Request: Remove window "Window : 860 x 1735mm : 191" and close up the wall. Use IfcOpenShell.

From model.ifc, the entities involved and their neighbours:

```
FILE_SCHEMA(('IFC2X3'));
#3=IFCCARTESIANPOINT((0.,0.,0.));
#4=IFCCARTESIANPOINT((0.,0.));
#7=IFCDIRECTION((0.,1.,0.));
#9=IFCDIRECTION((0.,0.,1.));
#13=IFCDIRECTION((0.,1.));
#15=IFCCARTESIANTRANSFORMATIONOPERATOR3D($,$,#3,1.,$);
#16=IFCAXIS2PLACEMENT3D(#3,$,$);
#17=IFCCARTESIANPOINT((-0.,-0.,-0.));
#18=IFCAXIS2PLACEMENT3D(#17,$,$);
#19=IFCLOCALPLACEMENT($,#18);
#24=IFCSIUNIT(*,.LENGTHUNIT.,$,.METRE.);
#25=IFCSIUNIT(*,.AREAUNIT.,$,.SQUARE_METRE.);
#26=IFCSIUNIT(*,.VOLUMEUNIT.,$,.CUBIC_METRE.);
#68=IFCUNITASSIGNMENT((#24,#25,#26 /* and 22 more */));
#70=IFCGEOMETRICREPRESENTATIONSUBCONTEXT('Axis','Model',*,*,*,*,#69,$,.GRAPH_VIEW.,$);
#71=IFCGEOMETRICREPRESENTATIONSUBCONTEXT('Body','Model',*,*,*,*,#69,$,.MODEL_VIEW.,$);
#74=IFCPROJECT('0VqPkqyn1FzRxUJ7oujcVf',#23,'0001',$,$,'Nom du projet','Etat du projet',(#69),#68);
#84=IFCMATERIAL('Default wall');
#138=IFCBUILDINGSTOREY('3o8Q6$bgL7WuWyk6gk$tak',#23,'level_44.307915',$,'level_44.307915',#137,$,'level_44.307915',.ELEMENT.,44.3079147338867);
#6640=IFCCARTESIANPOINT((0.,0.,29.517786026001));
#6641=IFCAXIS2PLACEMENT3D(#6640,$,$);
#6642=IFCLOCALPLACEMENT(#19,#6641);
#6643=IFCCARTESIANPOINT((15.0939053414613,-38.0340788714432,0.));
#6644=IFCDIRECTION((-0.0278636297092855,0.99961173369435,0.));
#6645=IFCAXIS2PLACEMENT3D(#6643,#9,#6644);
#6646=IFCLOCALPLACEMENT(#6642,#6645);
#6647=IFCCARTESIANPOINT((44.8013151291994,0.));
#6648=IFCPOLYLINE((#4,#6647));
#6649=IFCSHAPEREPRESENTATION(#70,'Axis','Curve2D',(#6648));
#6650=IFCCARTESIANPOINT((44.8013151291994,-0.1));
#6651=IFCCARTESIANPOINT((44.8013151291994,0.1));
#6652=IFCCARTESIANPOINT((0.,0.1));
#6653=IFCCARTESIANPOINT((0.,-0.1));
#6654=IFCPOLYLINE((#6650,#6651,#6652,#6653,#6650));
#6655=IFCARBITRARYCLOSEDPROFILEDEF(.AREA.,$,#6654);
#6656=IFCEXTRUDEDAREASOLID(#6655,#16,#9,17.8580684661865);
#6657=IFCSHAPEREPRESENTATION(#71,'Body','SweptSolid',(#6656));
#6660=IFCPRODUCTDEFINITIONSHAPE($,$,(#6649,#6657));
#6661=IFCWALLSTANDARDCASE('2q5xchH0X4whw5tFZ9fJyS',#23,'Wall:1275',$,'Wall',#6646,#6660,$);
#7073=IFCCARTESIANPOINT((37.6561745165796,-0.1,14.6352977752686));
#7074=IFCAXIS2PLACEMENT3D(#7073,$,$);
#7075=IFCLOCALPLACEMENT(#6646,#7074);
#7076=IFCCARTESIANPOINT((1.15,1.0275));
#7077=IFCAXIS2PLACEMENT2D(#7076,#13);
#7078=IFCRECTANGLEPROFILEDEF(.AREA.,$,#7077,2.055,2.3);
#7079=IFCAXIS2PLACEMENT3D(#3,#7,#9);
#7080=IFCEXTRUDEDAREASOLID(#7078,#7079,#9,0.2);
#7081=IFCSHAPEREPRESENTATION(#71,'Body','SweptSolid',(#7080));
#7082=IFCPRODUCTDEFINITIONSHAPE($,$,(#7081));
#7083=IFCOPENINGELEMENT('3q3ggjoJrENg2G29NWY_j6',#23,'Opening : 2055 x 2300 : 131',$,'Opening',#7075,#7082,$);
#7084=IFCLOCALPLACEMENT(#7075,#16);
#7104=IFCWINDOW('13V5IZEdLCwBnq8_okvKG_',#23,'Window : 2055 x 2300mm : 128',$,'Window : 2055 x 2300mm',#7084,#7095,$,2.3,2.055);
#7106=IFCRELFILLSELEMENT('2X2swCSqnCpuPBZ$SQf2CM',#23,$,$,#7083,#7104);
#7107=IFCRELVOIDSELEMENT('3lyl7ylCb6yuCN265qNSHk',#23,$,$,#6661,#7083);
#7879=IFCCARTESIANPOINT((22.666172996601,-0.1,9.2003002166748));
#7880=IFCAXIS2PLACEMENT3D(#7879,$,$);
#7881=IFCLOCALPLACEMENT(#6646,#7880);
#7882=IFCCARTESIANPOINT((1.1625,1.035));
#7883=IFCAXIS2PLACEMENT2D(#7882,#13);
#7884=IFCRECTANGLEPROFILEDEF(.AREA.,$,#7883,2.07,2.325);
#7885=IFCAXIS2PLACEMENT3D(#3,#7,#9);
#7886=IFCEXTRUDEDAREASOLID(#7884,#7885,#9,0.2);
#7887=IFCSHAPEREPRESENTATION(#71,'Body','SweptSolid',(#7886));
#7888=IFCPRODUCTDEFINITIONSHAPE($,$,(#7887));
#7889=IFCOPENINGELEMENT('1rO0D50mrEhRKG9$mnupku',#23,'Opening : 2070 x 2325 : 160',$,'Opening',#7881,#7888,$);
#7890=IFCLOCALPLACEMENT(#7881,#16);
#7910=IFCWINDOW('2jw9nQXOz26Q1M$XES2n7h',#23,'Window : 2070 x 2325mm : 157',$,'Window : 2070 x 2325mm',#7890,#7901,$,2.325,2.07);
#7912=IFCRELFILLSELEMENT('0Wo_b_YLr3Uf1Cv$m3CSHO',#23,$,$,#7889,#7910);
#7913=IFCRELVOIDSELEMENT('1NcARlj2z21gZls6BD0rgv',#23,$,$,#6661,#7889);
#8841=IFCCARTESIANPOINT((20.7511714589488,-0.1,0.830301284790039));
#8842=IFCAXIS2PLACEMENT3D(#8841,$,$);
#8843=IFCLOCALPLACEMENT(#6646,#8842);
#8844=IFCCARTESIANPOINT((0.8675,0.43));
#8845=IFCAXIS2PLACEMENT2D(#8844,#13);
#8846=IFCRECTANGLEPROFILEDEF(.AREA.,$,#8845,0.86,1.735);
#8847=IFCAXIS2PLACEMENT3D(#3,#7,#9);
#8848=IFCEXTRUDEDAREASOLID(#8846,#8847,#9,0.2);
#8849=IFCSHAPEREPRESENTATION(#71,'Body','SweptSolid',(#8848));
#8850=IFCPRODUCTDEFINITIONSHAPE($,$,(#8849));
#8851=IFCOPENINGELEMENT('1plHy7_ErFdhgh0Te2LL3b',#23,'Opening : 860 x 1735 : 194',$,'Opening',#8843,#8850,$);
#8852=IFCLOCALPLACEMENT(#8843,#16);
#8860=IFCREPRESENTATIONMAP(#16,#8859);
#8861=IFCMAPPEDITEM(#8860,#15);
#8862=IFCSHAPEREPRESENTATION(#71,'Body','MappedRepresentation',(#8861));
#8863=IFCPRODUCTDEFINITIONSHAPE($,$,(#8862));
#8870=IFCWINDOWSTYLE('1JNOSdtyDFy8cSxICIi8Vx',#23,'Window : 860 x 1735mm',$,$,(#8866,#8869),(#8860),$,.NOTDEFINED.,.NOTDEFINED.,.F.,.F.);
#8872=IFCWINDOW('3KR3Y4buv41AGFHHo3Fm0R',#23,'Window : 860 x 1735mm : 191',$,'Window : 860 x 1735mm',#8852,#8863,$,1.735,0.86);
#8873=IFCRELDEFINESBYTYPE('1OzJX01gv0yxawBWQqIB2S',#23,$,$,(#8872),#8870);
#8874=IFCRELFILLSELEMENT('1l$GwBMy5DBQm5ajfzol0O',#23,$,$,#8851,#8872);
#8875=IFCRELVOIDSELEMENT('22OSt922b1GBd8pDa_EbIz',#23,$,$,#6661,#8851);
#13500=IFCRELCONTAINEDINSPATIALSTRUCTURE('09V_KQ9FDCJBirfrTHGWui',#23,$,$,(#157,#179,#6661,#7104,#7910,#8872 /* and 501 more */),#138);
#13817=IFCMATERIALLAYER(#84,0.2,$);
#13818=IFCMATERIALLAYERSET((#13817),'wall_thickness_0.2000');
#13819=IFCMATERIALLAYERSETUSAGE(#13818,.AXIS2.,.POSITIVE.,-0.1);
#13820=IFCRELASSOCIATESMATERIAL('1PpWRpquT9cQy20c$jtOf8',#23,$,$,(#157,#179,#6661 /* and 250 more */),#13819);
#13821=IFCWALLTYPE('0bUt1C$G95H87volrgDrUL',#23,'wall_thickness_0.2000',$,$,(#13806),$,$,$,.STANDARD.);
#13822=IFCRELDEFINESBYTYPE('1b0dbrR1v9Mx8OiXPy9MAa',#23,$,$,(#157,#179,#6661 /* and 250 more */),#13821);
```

```python
import ifcopenshell
import ifcopenshell.api.feature
import ifcopenshell.api.root
import ifcopenshell.geom
import ifcopenshell.util.shape

model = ifcopenshell.open("model.ifc")
settings = ifcopenshell.geom.settings()


def volume(element):
    """Net volume in cubic metres, openings subtracted."""
    shape = ifcopenshell.geom.create_shape(settings, element)
    return ifcopenshell.util.shape.get_volume(shape.geometry)


window = model.by_guid("3KR3Y4buv41AGFHHo3Fm0R")
opening = window.FillsVoids[0].RelatingOpeningElement
wall = opening.VoidsElements[0].RelatingBuildingElement
before = volume(wall)

ifcopenshell.api.root.remove_product(model, product=window)
ifcopenshell.api.feature.remove_feature(model, feature=opening)

after = volume(wall)

print(f"wall volume {before:.3f} -> {after:.3f} m3")

model.write("model_v2.ifc")
```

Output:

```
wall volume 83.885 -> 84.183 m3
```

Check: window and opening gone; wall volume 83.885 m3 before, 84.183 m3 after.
